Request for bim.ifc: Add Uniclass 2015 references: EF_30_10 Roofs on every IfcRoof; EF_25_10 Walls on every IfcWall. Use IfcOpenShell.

First a look at what the model holds.

```python
import ifcopenshell

model = ifcopenshell.open("bim.ifc")
print(model.schema)
print("classifications:", [c.Name for c in model.by_type("IfcClassification")])
for ifc_class in ("IfcDoor", "IfcRoof", "IfcStair", "IfcWall", "IfcWindow"):
    print(ifc_class, len(model.by_type(ifc_class)))
```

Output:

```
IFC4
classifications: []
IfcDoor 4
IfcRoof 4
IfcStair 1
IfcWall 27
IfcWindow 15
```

```python
import ifcopenshell
import ifcopenshell.api.classification

model = ifcopenshell.open("bim.ifc")

system = ifcopenshell.api.classification.add_classification(model, classification="Uniclass 2015")

codes = {
    "IfcRoof": ("EF_30_10", "Roofs"),
    "IfcWall": ("EF_25_10", "Walls"),
}
for ifc_class, (code, name) in codes.items():
    products = model.by_type(ifc_class)
    ifcopenshell.api.classification.add_reference(
        model, products=products, classification=system, identification=code, name=name
    )
    print(code, len(products))

model.write("bim_rev.ifc")
```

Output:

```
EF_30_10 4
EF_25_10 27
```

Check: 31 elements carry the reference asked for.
